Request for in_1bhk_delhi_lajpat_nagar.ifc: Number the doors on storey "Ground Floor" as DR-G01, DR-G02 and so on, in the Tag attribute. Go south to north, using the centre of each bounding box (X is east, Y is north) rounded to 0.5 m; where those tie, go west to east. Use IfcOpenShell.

First a look at what the model holds.

```python
import ifcopenshell
import ifcopenshell.util.element
import ifcopenshell.util.placement

model = ifcopenshell.open("in_1bhk_delhi_lajpat_nagar.ifc")
print(model.schema)
storey = next(s for s in model.by_type("IfcBuildingStorey") if s.Name == "Ground Floor")
doors = [e for e in ifcopenshell.util.element.get_decomposition(storey) if e.is_a("IfcDoor")]
for e in sorted(doors, key=lambda e: e.id()):
    origin = ifcopenshell.util.placement.get_local_placement(e.ObjectPlacement)[:3, 3]
    print(e.id(), e.Tag, e.Name, origin.round(2) + 0.0, sep=" | ")
```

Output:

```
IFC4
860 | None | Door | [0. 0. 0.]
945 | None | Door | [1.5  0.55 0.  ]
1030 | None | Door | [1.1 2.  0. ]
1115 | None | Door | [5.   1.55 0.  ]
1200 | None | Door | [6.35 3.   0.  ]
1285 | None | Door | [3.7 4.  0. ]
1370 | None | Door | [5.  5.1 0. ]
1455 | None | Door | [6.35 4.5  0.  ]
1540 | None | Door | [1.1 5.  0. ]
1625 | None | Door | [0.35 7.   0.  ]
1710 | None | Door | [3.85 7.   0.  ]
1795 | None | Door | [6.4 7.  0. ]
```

```python
import ifcopenshell
import ifcopenshell.geom
import ifcopenshell.util.element
import ifcopenshell.util.shape

model = ifcopenshell.open("in_1bhk_delhi_lajpat_nagar.ifc")
settings = ifcopenshell.geom.settings()
settings.set("use-world-coords", True)


def centre(element):
    shape = ifcopenshell.geom.create_shape(settings, element)
    return ifcopenshell.util.shape.get_bbox_centroid(shape.geometry)


storey = next(s for s in model.by_type("IfcBuildingStorey") if s.Name == "Ground Floor")
doors = [e for e in ifcopenshell.util.element.get_decomposition(storey) if e.is_a("IfcDoor")]

# Insertion points can sit at a corner or the storey origin, so sort by the geometry (in metres).
centres = {e: centre(e) for e in doors}
doors.sort(key=lambda e: (round(centres[e][1] / 0.5), centres[e][0]))

for i, e in enumerate(doors, start=1):
    number = f"DR-G{i:02d}"
    e.Tag = number
    print(e.id(), number)

model.write("in_1bhk_delhi_lajpat_nagar_rev.ifc")
```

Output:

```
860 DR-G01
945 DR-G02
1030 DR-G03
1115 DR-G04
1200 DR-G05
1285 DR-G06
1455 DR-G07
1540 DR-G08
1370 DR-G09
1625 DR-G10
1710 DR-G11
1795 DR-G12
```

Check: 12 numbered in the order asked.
